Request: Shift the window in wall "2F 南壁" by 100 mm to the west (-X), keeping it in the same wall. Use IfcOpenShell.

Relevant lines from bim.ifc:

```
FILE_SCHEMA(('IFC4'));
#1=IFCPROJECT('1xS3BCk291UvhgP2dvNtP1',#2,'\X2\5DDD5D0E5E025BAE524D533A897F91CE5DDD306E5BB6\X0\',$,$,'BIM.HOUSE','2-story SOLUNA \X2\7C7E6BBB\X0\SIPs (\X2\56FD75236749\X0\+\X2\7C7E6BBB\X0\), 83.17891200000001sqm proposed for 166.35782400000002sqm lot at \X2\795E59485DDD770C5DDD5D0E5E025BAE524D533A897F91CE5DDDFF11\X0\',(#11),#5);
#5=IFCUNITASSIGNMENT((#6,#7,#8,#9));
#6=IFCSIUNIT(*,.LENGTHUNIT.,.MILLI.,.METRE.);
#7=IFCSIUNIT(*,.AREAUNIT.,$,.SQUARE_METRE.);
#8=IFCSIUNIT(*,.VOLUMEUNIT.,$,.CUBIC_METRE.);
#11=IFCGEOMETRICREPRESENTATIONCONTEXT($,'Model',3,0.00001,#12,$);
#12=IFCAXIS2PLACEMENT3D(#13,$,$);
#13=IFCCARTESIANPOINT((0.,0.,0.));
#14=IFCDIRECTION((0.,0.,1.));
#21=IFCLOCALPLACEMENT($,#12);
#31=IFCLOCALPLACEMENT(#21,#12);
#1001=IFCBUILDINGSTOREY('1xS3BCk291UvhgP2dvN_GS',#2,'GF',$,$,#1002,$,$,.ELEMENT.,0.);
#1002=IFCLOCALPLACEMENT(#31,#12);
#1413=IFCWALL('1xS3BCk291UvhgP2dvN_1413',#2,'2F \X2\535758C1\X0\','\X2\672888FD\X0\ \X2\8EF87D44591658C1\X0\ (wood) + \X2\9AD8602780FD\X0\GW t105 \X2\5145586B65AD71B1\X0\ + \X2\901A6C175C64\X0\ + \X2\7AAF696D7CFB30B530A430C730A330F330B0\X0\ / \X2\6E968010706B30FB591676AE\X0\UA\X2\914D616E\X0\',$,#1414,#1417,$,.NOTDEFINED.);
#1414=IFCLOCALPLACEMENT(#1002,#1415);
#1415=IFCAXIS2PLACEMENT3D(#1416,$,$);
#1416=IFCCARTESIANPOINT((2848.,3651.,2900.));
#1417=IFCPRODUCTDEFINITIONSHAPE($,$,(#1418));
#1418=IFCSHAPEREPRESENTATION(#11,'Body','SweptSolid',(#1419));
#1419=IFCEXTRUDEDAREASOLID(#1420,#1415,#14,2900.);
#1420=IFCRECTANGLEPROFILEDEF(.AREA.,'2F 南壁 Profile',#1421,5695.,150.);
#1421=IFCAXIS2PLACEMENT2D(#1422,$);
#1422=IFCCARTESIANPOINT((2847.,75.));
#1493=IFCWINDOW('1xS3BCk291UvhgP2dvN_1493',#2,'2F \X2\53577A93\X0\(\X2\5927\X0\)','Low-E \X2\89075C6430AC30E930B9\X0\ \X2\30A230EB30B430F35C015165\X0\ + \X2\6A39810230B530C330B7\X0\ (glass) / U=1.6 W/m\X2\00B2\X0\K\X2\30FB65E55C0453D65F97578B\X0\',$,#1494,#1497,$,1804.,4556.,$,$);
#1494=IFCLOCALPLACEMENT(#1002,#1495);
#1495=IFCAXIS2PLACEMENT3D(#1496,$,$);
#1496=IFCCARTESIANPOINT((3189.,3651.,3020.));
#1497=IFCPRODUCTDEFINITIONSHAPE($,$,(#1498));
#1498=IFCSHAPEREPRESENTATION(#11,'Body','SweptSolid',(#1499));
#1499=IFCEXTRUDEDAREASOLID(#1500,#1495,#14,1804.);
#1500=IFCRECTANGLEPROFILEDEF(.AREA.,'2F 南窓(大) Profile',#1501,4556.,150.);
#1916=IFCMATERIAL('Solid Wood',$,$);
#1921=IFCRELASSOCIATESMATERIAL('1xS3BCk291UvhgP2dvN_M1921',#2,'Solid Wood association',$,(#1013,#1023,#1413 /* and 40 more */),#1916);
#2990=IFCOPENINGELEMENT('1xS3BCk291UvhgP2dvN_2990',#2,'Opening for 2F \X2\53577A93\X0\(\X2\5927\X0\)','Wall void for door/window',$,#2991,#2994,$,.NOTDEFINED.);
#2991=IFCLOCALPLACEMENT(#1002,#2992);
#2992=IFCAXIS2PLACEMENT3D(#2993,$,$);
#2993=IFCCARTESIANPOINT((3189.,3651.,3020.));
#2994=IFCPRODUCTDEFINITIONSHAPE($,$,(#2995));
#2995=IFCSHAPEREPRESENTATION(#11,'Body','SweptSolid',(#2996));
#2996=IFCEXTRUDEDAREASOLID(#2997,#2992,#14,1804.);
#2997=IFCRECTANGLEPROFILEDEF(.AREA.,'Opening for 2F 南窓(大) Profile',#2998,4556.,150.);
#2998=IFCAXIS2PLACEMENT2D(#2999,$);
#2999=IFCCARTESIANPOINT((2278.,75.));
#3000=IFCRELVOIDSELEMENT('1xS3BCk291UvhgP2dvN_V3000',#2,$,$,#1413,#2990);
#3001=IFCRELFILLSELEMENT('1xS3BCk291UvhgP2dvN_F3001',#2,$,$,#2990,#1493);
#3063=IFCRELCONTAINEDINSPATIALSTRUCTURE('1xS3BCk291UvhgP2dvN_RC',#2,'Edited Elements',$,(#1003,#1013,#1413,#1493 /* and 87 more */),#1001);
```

```python
import ifcopenshell
import ifcopenshell.api.geometry
import ifcopenshell.util.placement

model = ifcopenshell.open("bim.ifc")

window = model.by_id(1493)
opening = window.FillsVoids[0].RelatingOpeningElement
wall = opening.VoidsElements[0].RelatingBuildingElement

wall_matrix = ifcopenshell.util.placement.get_local_placement(wall.ObjectPlacement)
shift = wall_matrix[:3, 0] * -100.0
before = ifcopenshell.util.placement.get_local_placement(window.ObjectPlacement)[:3, 3].copy()

# The window is not placed relative to its opening, so move both.
for product in (opening, window):
    matrix = ifcopenshell.util.placement.get_local_placement(product.ObjectPlacement)
    matrix[:3, 3] += shift
    ifcopenshell.api.geometry.edit_object_placement(model, product=product, matrix=matrix, is_si=False)

after = ifcopenshell.util.placement.get_local_placement(window.ObjectPlacement)[:3, 3]
print("window moved by", (after - before).round(3) + 0.0)

model.write("bim_rev.ifc")
```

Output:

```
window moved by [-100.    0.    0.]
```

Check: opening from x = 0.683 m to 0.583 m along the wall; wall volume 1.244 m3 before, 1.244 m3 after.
